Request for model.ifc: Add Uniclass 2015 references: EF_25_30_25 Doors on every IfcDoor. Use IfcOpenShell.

First a look at what the model holds.

```python
import ifcopenshell

model = ifcopenshell.open("model.ifc")
print(model.schema)
print("classifications:", [c.Name for c in model.by_type("IfcClassification")])
for ifc_class in ("IfcDoor", "IfcRoof", "IfcStair", "IfcWall", "IfcWindow"):
    print(ifc_class, len(model.by_type(ifc_class)))
```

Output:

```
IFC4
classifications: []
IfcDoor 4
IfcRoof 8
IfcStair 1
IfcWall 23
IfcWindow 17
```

```python
import ifcopenshell
import ifcopenshell.api.classification

model = ifcopenshell.open("model.ifc")

system = ifcopenshell.api.classification.add_classification(model, classification="Uniclass 2015")

codes = {
    "IfcDoor": ("EF_25_30_25", "Doors"),
}
for ifc_class, (code, name) in codes.items():
    products = model.by_type(ifc_class)
    ifcopenshell.api.classification.add_reference(
        model, products=products, classification=system, identification=code, name=name
    )
    print(code, len(products))

model.write("model-out.ifc")
```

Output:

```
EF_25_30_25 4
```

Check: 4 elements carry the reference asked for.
